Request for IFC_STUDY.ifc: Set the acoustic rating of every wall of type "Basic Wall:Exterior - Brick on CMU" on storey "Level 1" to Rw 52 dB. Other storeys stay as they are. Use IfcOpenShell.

First a look at what the model holds.

```python
import ifcopenshell
import ifcopenshell.util.element

model = ifcopenshell.open("IFC_STUDY.ifc")
print(model.schema)
storey = next(s for s in model.by_type("IfcBuildingStorey") if s.Name == "Level 1")
walls = [e for e in ifcopenshell.util.element.get_decomposition(storey) if e.is_a("IfcWall")]
seen = {}
for e in walls:
    element_type = ifcopenshell.util.element.get_type(e)
    key = (element_type.Name if element_type != e and element_type else None, ifcopenshell.util.element.get_pset(e, "Pset_WallCommon", "AcousticRating"))
    seen[key] = seen.get(key, 0) + 1
for (name, value), count in sorted(seen.items(), key=str):
    print(count, "x", name, "|", value)
```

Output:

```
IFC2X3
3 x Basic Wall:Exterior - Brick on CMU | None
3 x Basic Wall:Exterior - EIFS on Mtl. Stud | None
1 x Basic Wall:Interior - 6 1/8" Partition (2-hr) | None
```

```python
import ifcopenshell
import ifcopenshell.api.pset
import ifcopenshell.util.element

model = ifcopenshell.open("IFC_STUDY.ifc")

storey = next(s for s in model.by_type("IfcBuildingStorey") if s.Name == "Level 1")
walls = [e for e in ifcopenshell.util.element.get_decomposition(storey) if e.is_a("IfcWall")]

count = 0
for e in walls:
    element_type = ifcopenshell.util.element.get_type(e)
    if element_type in (None, e) or element_type.Name != "Basic Wall:Exterior - Brick on CMU":
        continue
    # add_pset returns the element's existing set when there is one.
    pset = ifcopenshell.api.pset.add_pset(model, product=e, name="Pset_WallCommon")
    ifcopenshell.api.pset.edit_pset(model, pset=pset, properties={"AcousticRating": "Rw 52 dB"})
    count += 1

print(count, "walls updated")

model.write("IFC_STUDY-out.ifc")
```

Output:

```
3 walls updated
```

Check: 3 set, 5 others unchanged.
